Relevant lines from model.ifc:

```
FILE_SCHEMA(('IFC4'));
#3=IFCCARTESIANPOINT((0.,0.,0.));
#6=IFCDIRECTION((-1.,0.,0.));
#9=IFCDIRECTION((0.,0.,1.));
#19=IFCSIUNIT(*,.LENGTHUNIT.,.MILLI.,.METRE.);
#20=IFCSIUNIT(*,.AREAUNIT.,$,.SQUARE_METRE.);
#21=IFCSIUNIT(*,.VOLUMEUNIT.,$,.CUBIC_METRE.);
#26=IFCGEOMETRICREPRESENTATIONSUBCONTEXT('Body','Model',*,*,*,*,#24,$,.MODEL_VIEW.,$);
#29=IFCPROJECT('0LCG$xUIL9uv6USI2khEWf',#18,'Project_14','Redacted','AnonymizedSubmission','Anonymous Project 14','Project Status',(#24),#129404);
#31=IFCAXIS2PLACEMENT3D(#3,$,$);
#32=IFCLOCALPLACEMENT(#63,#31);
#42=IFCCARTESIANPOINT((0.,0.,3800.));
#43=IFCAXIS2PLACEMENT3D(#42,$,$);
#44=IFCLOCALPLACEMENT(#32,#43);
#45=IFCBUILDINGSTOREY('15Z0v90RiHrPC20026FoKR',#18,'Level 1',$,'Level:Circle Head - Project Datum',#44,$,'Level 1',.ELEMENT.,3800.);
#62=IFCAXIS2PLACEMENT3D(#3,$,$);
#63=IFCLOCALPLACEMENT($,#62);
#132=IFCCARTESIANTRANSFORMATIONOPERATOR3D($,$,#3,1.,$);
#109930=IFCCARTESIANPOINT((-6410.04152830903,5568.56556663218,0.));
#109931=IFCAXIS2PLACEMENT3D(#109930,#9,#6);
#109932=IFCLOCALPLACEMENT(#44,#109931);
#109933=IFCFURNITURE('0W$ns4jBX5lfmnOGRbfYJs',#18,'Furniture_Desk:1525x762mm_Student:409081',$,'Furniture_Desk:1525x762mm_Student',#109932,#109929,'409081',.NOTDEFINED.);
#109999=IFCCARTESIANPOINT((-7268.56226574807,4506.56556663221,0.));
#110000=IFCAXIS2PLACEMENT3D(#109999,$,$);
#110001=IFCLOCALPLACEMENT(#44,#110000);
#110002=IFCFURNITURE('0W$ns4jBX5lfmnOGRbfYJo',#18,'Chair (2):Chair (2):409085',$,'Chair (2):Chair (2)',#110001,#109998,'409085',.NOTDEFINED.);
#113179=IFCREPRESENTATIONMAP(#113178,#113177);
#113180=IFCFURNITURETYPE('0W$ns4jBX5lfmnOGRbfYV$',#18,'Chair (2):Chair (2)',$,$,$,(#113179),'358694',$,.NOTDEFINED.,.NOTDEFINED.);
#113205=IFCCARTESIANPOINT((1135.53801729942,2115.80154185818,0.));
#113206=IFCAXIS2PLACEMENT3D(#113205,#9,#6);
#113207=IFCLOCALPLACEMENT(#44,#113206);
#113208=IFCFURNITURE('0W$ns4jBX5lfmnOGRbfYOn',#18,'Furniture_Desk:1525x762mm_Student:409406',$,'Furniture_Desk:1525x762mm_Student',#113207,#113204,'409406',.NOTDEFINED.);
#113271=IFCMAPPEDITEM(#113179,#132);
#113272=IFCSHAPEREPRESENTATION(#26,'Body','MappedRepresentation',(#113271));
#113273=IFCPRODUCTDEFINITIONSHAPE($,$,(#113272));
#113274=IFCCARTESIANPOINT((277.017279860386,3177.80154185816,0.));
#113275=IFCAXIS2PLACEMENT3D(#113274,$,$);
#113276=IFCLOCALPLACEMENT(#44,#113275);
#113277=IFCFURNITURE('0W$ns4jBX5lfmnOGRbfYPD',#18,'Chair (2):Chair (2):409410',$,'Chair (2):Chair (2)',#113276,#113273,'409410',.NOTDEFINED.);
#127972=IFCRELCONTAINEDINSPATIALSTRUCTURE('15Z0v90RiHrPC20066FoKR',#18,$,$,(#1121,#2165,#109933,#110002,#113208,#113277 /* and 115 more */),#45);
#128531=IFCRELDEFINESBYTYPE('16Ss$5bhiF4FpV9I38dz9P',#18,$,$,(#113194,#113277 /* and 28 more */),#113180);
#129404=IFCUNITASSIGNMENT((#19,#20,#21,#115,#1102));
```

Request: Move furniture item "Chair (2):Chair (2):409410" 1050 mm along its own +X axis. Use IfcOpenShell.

```python
import ifcopenshell
import ifcopenshell.api.geometry
import ifcopenshell.util.placement

model = ifcopenshell.open("model.ifc")

item = model.by_id(113277)
matrix = ifcopenshell.util.placement.get_local_placement(item.ObjectPlacement)
matrix[:3, 3] += matrix[:3, 0] * 1050.0
ifcopenshell.api.geometry.edit_object_placement(model, product=item, matrix=matrix, is_si=False)

print(ifcopenshell.util.placement.get_local_placement(item.ObjectPlacement).round(3) + 0.0)

model.write("model_updated.ifc")
```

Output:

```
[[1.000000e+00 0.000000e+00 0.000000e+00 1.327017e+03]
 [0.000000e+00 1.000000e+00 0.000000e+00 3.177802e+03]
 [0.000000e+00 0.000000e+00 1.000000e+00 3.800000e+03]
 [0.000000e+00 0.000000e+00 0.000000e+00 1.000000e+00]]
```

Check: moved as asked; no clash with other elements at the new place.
